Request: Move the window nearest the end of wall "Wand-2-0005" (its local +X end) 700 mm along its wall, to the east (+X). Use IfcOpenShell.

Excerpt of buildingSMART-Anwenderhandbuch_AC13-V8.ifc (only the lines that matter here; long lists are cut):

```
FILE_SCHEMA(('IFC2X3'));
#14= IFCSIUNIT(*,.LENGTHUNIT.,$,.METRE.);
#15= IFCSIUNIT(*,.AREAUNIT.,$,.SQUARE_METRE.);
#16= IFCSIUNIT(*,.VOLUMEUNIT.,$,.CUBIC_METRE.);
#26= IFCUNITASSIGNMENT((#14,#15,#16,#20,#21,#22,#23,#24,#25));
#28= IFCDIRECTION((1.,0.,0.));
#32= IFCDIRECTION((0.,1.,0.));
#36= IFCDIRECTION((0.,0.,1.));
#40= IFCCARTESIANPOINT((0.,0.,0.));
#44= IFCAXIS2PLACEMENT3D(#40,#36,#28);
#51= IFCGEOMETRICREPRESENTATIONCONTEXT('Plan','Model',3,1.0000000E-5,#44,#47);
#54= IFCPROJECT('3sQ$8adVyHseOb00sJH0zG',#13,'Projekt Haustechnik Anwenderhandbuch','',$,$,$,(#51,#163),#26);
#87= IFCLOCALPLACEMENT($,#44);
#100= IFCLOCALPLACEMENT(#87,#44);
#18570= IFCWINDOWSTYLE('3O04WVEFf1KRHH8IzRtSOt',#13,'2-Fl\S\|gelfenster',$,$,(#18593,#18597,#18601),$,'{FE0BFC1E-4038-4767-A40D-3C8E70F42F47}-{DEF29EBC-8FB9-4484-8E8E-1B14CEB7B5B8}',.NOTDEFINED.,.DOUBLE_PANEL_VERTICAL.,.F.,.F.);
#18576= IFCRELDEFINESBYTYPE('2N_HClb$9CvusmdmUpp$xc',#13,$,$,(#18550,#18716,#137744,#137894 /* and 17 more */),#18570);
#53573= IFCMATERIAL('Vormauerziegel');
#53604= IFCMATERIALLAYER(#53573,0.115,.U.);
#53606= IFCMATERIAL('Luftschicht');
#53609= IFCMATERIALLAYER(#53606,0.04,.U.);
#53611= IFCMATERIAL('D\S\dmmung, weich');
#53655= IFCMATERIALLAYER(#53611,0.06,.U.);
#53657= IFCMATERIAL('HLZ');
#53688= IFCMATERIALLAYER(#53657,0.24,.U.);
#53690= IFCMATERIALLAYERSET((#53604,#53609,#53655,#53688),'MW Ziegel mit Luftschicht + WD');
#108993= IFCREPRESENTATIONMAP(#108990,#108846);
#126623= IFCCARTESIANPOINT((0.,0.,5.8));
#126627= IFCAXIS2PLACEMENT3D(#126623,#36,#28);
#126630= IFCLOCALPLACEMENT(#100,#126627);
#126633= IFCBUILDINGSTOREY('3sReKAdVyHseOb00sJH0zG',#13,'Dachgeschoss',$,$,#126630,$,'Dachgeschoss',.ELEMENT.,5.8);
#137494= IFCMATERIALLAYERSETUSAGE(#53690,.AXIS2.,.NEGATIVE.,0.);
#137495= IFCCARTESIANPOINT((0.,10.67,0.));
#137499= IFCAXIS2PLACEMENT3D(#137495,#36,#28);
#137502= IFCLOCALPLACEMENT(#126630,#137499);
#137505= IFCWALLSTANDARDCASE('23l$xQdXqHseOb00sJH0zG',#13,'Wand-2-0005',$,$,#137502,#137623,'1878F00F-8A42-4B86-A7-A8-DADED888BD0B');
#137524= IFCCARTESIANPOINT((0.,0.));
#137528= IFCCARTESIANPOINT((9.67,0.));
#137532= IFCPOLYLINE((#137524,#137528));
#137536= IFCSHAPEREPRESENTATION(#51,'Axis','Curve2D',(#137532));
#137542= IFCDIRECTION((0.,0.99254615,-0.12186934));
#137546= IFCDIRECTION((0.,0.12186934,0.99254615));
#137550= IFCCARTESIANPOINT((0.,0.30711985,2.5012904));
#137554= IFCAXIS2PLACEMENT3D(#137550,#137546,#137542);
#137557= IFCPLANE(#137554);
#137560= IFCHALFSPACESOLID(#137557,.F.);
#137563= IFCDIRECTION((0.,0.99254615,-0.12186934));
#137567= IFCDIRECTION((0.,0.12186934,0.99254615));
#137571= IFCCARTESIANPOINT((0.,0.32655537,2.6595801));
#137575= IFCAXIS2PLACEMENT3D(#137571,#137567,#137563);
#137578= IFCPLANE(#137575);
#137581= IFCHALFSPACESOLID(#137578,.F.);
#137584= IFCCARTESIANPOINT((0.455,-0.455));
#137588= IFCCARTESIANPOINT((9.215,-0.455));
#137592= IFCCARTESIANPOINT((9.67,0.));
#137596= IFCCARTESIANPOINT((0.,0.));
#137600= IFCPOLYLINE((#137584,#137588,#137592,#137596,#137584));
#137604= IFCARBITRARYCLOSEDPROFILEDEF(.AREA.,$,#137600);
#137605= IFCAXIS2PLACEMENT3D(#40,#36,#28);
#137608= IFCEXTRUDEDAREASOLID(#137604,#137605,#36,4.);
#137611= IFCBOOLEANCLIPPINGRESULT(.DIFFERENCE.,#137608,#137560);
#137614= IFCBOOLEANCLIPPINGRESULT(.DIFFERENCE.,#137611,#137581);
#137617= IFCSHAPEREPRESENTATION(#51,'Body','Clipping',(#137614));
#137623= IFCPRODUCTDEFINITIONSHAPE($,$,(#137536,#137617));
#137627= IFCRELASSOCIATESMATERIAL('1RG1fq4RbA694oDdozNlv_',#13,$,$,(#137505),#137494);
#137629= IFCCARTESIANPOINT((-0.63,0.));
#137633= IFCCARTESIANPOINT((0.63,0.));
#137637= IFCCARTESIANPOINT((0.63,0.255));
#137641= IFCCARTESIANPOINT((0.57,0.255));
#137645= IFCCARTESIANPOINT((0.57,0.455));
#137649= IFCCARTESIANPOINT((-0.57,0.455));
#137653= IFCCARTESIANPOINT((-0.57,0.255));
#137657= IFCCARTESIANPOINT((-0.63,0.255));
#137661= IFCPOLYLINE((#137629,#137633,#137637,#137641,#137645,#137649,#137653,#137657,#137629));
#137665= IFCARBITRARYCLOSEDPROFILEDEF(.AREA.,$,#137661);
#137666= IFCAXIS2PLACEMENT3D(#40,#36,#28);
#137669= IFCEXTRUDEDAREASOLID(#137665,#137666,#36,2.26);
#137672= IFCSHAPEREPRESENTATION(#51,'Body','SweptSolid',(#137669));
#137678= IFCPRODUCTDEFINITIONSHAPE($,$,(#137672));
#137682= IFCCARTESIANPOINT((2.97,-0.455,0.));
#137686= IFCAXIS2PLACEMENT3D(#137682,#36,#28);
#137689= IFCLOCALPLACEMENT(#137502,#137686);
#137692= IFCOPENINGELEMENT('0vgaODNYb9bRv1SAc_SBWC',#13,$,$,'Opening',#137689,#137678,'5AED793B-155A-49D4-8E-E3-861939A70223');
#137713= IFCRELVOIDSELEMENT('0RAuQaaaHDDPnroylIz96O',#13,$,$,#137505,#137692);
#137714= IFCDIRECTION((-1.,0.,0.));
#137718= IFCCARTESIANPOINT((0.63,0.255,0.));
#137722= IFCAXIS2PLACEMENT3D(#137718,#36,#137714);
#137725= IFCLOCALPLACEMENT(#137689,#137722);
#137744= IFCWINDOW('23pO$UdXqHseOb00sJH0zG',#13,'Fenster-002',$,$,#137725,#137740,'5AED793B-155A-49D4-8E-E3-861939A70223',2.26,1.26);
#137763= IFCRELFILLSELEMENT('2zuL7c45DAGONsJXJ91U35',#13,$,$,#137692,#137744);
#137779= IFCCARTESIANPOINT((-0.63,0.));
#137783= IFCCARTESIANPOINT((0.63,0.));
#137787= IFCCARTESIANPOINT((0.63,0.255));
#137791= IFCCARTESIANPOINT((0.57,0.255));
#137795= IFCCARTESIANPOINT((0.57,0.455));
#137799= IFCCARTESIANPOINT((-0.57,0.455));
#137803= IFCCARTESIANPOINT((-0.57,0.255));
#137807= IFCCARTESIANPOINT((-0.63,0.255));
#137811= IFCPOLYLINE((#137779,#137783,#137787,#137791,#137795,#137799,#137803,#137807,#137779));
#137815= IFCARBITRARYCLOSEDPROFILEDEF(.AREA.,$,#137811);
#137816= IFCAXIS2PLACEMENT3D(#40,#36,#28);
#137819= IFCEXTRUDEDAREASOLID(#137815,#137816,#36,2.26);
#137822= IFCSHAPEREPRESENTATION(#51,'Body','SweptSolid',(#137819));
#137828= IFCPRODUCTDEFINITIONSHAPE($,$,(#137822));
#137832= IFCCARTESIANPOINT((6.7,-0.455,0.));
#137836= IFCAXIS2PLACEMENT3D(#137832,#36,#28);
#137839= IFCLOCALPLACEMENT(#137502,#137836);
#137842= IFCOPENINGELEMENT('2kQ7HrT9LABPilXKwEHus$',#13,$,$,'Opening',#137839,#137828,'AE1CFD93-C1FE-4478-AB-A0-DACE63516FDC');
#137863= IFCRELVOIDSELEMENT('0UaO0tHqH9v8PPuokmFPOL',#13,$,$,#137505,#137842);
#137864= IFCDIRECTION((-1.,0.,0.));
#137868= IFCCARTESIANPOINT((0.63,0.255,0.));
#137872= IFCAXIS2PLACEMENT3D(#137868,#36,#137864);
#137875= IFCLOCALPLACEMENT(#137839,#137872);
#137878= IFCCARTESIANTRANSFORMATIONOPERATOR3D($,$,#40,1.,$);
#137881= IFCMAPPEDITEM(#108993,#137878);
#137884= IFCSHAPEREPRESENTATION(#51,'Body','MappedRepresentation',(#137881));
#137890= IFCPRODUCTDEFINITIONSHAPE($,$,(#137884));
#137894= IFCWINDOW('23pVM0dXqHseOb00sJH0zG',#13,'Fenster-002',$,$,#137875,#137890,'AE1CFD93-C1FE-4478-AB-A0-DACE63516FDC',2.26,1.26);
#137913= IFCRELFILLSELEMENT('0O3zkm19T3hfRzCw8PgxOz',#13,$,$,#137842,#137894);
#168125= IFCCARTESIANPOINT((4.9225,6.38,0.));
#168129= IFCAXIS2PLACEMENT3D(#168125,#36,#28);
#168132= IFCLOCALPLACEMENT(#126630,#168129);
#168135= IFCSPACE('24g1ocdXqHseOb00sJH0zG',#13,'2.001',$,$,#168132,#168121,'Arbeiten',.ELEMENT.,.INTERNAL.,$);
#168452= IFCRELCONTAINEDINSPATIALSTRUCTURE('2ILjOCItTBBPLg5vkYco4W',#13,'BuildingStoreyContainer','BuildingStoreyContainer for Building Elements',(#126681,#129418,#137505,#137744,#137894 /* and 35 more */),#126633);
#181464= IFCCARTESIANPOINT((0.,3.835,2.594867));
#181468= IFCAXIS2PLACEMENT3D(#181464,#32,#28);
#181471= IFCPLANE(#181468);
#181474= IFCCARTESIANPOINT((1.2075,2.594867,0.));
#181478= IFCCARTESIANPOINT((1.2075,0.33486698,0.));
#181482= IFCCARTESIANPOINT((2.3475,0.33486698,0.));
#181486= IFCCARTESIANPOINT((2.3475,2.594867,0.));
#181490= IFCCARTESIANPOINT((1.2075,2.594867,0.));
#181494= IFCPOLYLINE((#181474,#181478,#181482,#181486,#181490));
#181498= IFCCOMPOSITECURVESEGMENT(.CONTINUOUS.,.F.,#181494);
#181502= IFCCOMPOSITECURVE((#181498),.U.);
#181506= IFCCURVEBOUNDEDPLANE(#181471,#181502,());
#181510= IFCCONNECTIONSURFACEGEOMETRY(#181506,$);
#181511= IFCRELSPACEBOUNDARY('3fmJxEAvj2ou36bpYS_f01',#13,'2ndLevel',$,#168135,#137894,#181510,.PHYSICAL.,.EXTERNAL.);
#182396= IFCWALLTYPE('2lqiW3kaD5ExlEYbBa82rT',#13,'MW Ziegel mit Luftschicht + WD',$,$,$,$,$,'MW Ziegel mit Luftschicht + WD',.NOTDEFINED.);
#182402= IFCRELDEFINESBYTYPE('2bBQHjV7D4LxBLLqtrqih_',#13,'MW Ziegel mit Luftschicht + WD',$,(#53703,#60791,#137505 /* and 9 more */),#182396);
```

```python
import numpy as np
import ifcopenshell
import ifcopenshell.api.geometry
import ifcopenshell.util.placement
import ifcopenshell.util.unit

model = ifcopenshell.open("buildingSMART-Anwenderhandbuch_AC13-V8.ifc")
unit_scale = ifcopenshell.util.unit.calculate_unit_scale(model)

window = model.by_guid("23pVM0dXqHseOb00sJH0zG")
opening = window.FillsVoids[0].RelatingOpeningElement
wall = opening.VoidsElements[0].RelatingBuildingElement

wall_matrix = ifcopenshell.util.placement.get_local_placement(wall.ObjectPlacement)
shift = wall_matrix[:3, 0] * 0.7 / unit_scale
before = ifcopenshell.util.placement.get_local_placement(window.ObjectPlacement)[:3, 3].copy()

# The window is placed relative to its opening, so it follows when the opening moves.
matrix = ifcopenshell.util.placement.get_local_placement(opening.ObjectPlacement)
matrix[:3, 3] += shift
ifcopenshell.api.geometry.edit_object_placement(
    model, product=opening, matrix=matrix, is_si=False, should_transform_children=True
)

# Space boundary surfaces are stored in each space's coordinates; move them too.
for rel in window.ProvidesBoundaries:
    if not rel.ConnectionGeometry:
        continue
    surface = rel.ConnectionGeometry.SurfaceOnRelatingElement.BasisSurface
    space_matrix = ifcopenshell.util.placement.get_local_placement(rel.RelatingSpace.ObjectPlacement)
    point = np.array(surface.Position.Location.Coordinates) + space_matrix[:3, :3].T @ shift
    surface.Position = model.createIfcAxis2Placement3D(
        model.createIfcCartesianPoint(point.tolist()), surface.Position.Axis, surface.Position.RefDirection
    )

after = ifcopenshell.util.placement.get_local_placement(window.ObjectPlacement)[:3, 3]
print("window moved by", (after - before).round(3) + 0.0)

model.write("buildingSMART-Anwenderhandbuch_AC13-V8_rev.ifc")
```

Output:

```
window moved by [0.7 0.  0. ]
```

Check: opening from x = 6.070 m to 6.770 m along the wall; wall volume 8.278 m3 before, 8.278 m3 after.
